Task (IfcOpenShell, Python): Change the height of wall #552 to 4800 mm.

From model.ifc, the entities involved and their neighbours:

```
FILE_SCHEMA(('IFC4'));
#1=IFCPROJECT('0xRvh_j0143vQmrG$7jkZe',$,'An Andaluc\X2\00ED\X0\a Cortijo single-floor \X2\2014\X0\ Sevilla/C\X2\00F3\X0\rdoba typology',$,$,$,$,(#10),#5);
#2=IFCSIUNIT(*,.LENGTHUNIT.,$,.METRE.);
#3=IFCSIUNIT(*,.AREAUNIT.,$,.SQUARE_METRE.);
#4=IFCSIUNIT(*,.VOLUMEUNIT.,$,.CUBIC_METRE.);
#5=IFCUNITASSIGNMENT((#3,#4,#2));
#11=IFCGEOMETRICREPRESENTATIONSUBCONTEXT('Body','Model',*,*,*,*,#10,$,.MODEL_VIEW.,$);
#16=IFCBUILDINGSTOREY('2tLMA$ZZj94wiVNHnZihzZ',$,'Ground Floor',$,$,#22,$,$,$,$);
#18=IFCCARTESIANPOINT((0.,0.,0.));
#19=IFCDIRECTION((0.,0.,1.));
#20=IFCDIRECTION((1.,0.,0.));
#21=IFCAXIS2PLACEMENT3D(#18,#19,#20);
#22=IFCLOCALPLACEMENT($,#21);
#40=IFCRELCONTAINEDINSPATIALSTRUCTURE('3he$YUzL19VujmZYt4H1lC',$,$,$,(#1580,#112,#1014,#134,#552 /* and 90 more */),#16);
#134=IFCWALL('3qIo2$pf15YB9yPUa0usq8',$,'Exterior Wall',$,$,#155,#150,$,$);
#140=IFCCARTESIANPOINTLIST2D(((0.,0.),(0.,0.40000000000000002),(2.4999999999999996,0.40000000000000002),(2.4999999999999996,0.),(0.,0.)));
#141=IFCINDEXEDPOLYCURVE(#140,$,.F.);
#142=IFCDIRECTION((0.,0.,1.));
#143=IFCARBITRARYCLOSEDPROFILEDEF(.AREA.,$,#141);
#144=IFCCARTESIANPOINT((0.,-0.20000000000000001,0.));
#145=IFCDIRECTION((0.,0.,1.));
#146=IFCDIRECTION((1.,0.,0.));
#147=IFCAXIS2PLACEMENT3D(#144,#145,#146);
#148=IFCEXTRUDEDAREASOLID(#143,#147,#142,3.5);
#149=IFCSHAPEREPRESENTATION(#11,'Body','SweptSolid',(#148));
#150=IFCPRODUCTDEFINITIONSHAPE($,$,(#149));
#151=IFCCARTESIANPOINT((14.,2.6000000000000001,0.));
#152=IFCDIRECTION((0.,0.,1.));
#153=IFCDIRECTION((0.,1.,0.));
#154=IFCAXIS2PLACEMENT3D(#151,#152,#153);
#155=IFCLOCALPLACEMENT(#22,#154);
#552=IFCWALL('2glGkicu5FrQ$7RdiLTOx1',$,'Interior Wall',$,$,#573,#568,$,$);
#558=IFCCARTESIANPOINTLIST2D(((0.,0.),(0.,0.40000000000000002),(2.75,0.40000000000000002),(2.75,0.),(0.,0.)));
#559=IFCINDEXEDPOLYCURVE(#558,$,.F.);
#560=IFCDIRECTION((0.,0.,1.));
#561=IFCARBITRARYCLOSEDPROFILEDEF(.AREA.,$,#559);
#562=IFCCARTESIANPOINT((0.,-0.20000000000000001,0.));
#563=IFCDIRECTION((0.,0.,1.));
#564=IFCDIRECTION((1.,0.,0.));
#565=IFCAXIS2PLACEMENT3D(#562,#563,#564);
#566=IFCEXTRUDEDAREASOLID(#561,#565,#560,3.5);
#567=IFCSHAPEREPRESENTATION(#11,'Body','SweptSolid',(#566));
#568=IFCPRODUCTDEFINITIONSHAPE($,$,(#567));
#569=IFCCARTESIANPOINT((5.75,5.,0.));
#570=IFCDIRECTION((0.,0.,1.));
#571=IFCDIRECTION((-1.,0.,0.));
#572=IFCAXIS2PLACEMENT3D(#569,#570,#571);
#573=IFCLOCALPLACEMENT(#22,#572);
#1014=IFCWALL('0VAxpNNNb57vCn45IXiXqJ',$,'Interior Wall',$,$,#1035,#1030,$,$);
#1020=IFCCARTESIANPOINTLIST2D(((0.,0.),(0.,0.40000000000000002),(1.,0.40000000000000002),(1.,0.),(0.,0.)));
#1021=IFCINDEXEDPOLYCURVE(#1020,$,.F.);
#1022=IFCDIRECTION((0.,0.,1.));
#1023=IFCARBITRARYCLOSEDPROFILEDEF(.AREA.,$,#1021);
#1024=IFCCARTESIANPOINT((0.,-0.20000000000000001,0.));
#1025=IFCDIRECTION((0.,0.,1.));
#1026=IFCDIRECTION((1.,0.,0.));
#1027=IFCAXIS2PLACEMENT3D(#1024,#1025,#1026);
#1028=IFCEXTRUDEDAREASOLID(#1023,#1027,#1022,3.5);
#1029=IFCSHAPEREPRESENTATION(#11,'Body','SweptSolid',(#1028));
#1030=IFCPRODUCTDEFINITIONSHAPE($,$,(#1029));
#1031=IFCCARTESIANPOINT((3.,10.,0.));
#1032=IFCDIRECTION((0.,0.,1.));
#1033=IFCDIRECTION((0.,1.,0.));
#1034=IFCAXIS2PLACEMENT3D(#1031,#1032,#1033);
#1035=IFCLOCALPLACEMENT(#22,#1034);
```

```python
import ifcopenshell
import ifcopenshell.geom
import ifcopenshell.util.representation
import ifcopenshell.util.shape

model = ifcopenshell.open("model.ifc")
settings = ifcopenshell.geom.settings()


def volume(element):
    """Net volume in cubic metres, openings subtracted."""
    shape = ifcopenshell.geom.create_shape(settings, element)
    return ifcopenshell.util.shape.get_volume(shape.geometry)


wall = model.by_id(552)
before = volume(wall)

body = ifcopenshell.util.representation.get_representation(wall, "Model", "Body")
solid = body.Items[0]
old_height = solid.Depth
solid.Depth = 4.8
after = volume(wall)

print(f"height {old_height:g} -> {solid.Depth:g}, volume {before:.3f} -> {after:.3f} m3")

model.write("model_v2.ifc")
```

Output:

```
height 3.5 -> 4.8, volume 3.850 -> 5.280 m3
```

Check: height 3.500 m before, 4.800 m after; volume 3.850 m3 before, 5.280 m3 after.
